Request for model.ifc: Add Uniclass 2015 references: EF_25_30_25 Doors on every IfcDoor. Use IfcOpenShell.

First a look at what the model holds.

```python
import ifcopenshell

model = ifcopenshell.open("model.ifc")
print(model.schema)
print("classifications:", [c.Name for c in model.by_type("IfcClassification")])
for ifc_class in ("IfcDoor", "IfcRoof", "IfcStair", "IfcWall", "IfcWindow"):
    print(ifc_class, len(model.by_type(ifc_class)))
```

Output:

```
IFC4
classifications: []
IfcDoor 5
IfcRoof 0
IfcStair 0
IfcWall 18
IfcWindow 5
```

```python
import ifcopenshell
import ifcopenshell.api.classification

model = ifcopenshell.open("model.ifc")

system = ifcopenshell.api.classification.add_classification(model, classification="Uniclass 2015")

codes = {
    "IfcDoor": ("EF_25_30_25", "Doors"),
}
for ifc_class, (code, name) in codes.items():
    products = model.by_type(ifc_class)
    ifcopenshell.api.classification.add_reference(
        model, products=products, classification=system, identification=code, name=name
    )
    print(code, len(products))

model.write("model_updated.ifc")
```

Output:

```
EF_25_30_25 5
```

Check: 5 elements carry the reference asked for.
